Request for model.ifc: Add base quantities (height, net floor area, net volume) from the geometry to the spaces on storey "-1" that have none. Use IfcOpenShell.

First a look at what the model holds.

```python
import ifcopenshell
import ifcopenshell.util.element
import ifcopenshell.util.unit

model = ifcopenshell.open("model.ifc")
print(model.schema)
for unit_type in ("LENGTHUNIT", "AREAUNIT", "VOLUMEUNIT"):
    print(unit_type, ifcopenshell.util.unit.calculate_unit_scale(model, unit_type))
storey = next(s for s in model.by_type("IfcBuildingStorey") if s.Name == "-1")
spaces = [e for e in ifcopenshell.util.element.get_decomposition(storey) if e.is_a("IfcSpace")]
for e in sorted(spaces, key=lambda e: e.id()):
    print(e.id(), e.is_a(), e.Name, list(ifcopenshell.util.element.get_psets(e, qtos_only=True)), sep=" | ")
```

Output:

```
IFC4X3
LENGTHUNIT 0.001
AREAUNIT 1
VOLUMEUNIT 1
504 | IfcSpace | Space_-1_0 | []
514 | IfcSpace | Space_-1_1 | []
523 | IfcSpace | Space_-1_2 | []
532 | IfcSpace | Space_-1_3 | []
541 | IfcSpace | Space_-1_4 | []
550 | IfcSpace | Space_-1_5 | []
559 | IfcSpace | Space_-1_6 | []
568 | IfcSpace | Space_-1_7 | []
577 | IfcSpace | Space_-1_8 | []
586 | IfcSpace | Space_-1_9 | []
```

```python
import ifcopenshell
import ifcopenshell.api.pset
import ifcopenshell.geom
import ifcopenshell.util.element
import ifcopenshell.util.shape
import ifcopenshell.util.unit

model = ifcopenshell.open("model.ifc")
unit_scale = ifcopenshell.util.unit.calculate_unit_scale(model)
area_scale = ifcopenshell.util.unit.calculate_unit_scale(model, "AREAUNIT")
volume_scale = ifcopenshell.util.unit.calculate_unit_scale(model, "VOLUMEUNIT")
settings = ifcopenshell.geom.settings()

storey = next(s for s in model.by_type("IfcBuildingStorey") if s.Name == "-1")
spaces = [e for e in ifcopenshell.util.element.get_decomposition(storey) if e.is_a("IfcSpace")]

for e in sorted(spaces, key=lambda e: e.id()):
    if ifcopenshell.util.element.get_psets(e, qtos_only=True, should_inherit=False):
        continue
    # Geometry comes back in metres, in the element's own axes.
    shape = ifcopenshell.geom.create_shape(settings, e)
    values = {
        "Height": ifcopenshell.util.shape.get_z(shape.geometry) / unit_scale,
        "NetFloorArea": ifcopenshell.util.shape.get_footprint_area(shape.geometry) / area_scale,
        "NetVolume": ifcopenshell.util.shape.get_volume(shape.geometry) / volume_scale,
    }
    qto = ifcopenshell.api.pset.add_qto(model, product=e, name="Qto_SpaceBaseQuantities")
    ifcopenshell.api.pset.edit_qto(model, qto=qto, properties=values)
    print(e.id(), {k: round(v, 3) for k, v in values.items()})

model.write("model_edited.ifc")
```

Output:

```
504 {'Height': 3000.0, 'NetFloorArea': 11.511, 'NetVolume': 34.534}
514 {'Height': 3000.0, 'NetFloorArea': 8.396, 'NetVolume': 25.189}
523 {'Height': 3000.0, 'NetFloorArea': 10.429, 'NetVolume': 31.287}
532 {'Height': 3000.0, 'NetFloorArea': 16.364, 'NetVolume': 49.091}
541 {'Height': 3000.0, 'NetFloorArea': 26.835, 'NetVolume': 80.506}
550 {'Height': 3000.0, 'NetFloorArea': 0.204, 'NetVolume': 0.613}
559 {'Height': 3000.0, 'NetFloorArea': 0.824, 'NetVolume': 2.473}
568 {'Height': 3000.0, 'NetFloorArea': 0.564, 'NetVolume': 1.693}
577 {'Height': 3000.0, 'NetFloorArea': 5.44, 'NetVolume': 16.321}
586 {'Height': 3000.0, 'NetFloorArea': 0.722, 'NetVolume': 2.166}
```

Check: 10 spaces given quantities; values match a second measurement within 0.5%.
